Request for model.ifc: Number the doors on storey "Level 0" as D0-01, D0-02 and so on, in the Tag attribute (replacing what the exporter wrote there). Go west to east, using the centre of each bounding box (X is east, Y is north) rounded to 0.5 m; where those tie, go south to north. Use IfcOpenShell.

First a look at what the model holds.

```python
import ifcopenshell
import ifcopenshell.util.element
import ifcopenshell.util.placement

model = ifcopenshell.open("model.ifc")
print(model.schema)
storey = next(s for s in model.by_type("IfcBuildingStorey") if s.Name == "Level 0")
doors = [e for e in ifcopenshell.util.element.get_decomposition(storey) if e.is_a("IfcDoor")]
for e in sorted(doors, key=lambda e: e.id()):
    origin = ifcopenshell.util.placement.get_local_placement(e.ObjectPlacement)[:3, 3]
    print(e.id(), e.Tag, e.Name, origin.round(2) + 0.0, sep=" | ")
```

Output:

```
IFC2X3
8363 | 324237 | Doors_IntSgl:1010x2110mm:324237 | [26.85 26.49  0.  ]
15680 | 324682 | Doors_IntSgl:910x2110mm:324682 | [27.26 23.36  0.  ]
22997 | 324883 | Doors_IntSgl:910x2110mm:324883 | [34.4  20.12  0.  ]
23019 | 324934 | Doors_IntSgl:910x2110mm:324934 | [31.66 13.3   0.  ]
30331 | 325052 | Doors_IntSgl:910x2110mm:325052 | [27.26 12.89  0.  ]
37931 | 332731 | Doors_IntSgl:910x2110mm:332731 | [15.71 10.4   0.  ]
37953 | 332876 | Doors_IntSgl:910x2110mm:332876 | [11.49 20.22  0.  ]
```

```python
import ifcopenshell
import ifcopenshell.geom
import ifcopenshell.util.element
import ifcopenshell.util.shape

model = ifcopenshell.open("model.ifc")
settings = ifcopenshell.geom.settings()
settings.set("use-world-coords", True)


def centre(element):
    shape = ifcopenshell.geom.create_shape(settings, element)
    return ifcopenshell.util.shape.get_bbox_centroid(shape.geometry)


storey = next(s for s in model.by_type("IfcBuildingStorey") if s.Name == "Level 0")
doors = [e for e in ifcopenshell.util.element.get_decomposition(storey) if e.is_a("IfcDoor")]

# Insertion points can sit at a corner or the storey origin, so sort by the geometry (in metres).
centres = {e: centre(e) for e in doors}
doors.sort(key=lambda e: (round(centres[e][0] / 0.5), centres[e][1]))

for i, e in enumerate(doors, start=1):
    number = f"D0-{i:02d}"
    e.Tag = number
    print(e.id(), number)

model.write("model_edited.ifc")
```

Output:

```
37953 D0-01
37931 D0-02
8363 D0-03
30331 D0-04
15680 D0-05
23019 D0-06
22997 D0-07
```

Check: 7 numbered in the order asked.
